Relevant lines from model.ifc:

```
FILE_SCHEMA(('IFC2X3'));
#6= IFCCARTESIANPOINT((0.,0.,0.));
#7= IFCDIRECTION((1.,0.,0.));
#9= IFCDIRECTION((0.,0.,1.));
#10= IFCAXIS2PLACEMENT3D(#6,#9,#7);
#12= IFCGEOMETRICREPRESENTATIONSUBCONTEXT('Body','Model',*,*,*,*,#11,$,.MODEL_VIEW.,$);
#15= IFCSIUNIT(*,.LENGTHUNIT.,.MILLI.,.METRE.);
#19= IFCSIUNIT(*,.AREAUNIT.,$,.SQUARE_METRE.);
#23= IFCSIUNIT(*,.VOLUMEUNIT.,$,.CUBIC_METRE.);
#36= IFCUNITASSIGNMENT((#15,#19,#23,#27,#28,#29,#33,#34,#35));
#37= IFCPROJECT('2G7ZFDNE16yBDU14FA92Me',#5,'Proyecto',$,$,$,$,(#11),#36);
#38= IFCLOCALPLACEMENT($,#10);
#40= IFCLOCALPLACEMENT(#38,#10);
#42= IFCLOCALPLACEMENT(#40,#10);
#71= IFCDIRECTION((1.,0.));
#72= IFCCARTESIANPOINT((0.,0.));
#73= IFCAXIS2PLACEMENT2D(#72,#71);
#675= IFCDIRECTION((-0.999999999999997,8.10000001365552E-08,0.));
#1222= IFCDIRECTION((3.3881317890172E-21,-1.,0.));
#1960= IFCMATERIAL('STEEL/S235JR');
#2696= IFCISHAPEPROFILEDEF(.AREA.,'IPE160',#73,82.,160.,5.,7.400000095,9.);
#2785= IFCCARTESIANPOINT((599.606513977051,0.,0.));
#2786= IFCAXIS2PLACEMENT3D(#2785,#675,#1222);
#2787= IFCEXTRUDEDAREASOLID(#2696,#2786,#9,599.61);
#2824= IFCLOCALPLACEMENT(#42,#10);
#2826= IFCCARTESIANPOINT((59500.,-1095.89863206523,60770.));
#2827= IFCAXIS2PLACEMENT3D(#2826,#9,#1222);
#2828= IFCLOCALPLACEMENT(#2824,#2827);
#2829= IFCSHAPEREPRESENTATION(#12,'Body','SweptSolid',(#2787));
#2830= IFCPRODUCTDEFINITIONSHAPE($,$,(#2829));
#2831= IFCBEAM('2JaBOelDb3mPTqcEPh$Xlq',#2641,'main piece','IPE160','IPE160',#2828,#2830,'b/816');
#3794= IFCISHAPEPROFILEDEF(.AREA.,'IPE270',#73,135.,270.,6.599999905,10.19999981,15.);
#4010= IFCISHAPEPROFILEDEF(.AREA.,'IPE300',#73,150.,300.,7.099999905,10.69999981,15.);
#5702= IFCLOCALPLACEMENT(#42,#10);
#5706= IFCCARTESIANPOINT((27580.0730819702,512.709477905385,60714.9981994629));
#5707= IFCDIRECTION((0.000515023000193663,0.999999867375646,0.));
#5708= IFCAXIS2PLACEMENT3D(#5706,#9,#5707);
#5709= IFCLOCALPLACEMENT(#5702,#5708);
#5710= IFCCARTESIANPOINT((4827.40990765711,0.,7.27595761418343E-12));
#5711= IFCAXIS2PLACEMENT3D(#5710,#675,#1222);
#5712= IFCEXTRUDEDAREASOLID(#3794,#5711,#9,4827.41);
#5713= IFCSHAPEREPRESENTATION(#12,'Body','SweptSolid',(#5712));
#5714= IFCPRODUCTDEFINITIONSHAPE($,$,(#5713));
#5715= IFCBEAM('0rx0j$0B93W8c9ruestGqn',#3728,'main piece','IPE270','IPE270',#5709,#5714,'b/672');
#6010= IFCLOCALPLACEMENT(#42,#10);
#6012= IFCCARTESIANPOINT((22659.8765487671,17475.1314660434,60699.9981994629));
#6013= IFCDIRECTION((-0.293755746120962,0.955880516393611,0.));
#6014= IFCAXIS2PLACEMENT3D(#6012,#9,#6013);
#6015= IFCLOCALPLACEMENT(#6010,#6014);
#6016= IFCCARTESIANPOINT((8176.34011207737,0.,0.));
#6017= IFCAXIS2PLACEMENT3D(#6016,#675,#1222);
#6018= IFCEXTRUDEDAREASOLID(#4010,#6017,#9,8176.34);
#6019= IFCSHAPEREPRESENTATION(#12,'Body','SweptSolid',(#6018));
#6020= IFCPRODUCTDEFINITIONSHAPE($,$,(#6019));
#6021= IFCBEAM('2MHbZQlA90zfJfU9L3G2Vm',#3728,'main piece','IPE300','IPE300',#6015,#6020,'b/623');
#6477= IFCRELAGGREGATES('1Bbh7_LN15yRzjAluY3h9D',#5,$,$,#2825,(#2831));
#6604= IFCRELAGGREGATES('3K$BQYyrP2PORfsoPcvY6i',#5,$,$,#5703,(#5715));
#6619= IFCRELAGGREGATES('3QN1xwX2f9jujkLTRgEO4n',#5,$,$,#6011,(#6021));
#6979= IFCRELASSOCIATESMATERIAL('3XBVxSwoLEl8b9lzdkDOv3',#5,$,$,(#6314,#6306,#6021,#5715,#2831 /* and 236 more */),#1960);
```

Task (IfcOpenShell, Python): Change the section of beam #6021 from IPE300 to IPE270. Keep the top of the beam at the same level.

```python
import ifcopenshell
import ifcopenshell.util.element
import ifcopenshell.util.representation

model = ifcopenshell.open("model.ifc")

member = model.by_guid("2MHbZQlA90zfJfU9L3G2Vm")
source = next(p for p in model.by_type("IfcIShapeProfileDef") if p.ProfileName == "IPE270")

body = ifcopenshell.util.representation.get_representation(member, "Model", "Body")
solid = body.Items[0]
old_profile = solid.SweptArea

# Copy the section's sizes but keep this member's own profile position.
profile = ifcopenshell.util.element.copy(model, source)
# Profiles are centred, so shift by half the change in depth to hold the top.
shift = (old_profile.OverallDepth - profile.OverallDepth) / 2
x, y = old_profile.Position.Location.Coordinates
up = (0.0, 1.0)  # upwards, in the solid's own plane
location = model.createIfcCartesianPoint((x + up[0] * shift, y + up[1] * shift))
profile.Position = model.createIfcAxis2Placement2D(location, old_profile.Position.RefDirection)
solid.SweptArea = profile
if not model.get_total_inverses(old_profile):
    ifcopenshell.util.element.remove_deep2(model, old_profile)
member.Description = member.Description.replace("IPE300", "IPE270")
member.ObjectType = member.ObjectType.replace("IPE300", "IPE270")

print(solid.SweptArea)

model.write("model_v2.ifc")
```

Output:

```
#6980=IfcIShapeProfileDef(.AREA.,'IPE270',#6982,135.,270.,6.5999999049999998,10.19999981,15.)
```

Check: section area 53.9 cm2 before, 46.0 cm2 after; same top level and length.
